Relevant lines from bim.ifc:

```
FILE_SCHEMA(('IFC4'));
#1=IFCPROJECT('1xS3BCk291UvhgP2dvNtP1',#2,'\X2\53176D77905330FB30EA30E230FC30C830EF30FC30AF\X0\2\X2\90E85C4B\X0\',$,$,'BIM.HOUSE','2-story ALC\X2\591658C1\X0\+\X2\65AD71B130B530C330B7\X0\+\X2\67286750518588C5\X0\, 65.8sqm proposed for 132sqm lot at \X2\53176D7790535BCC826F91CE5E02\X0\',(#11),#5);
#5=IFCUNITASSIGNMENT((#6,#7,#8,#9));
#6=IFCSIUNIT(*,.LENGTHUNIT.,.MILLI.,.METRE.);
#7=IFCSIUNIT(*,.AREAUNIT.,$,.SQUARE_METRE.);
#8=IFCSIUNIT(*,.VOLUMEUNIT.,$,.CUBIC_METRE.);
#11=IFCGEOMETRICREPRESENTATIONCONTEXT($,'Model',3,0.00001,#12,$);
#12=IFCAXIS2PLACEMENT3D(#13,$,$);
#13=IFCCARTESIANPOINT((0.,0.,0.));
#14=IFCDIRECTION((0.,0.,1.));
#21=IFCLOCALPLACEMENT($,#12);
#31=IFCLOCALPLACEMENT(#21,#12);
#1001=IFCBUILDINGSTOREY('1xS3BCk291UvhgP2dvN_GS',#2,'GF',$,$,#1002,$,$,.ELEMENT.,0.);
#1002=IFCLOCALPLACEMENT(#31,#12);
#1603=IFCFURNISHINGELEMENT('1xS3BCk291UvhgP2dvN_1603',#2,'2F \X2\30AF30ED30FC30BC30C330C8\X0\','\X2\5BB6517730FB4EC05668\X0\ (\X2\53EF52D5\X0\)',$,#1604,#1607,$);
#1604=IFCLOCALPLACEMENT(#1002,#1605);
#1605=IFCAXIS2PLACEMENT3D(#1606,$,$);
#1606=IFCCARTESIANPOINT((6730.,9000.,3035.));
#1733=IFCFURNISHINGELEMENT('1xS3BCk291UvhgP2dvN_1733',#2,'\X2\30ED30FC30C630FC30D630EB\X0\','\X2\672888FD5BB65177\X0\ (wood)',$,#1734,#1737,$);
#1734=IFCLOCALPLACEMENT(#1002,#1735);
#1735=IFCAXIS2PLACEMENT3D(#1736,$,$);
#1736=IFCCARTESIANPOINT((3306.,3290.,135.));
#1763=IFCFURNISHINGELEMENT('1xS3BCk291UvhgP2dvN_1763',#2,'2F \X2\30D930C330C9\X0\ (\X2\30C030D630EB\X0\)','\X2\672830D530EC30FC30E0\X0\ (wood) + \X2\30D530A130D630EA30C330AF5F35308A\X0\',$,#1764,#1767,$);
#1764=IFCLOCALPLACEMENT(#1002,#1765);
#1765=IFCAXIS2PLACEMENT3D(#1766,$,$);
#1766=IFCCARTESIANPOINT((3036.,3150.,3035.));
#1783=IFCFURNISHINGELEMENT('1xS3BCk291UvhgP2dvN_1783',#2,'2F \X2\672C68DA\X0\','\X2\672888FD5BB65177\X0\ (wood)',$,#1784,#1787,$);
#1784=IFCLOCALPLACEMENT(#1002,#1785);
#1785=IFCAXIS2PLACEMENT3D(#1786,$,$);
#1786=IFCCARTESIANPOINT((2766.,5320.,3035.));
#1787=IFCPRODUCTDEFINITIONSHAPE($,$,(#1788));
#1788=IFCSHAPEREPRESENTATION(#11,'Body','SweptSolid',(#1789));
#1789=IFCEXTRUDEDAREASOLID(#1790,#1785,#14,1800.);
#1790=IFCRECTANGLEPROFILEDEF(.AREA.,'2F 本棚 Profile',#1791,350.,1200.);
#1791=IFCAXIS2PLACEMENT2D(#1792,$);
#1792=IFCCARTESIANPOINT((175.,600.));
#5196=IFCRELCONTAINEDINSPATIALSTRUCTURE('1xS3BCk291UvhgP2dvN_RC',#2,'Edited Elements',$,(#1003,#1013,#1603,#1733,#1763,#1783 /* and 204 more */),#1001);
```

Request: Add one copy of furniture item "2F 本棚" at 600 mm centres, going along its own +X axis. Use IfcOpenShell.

```python
import ifcopenshell
import ifcopenshell.api.geometry
import ifcopenshell.api.root
import ifcopenshell.util.element
import ifcopenshell.util.placement
import ifcopenshell.util.unit

model = ifcopenshell.open("bim.ifc")
unit_scale = ifcopenshell.util.unit.calculate_unit_scale(model)


def reuse_history(source, copy):
    """copy_class also copies each property set's owner history, people and application; keep the originals."""
    for rel in copy.IsDefinedBy:
        if rel.is_a("IfcRelDefinesByProperties") and (history := rel.RelatingPropertyDefinition.OwnerHistory):
            rel.RelatingPropertyDefinition.OwnerHistory = source.OwnerHistory
            ifcopenshell.util.element.remove_deep2(model, history)


source = model.by_guid("1xS3BCk291UvhgP2dvN_1783")
base = ifcopenshell.util.placement.get_local_placement(source.ObjectPlacement)
step = base[:3, 0] * 0.6 / unit_scale

for i in range(1, 2):
    copy = ifcopenshell.api.root.copy_class(model, product=source)
    copy.Representation = ifcopenshell.util.element.copy_deep(
        model, source.Representation, exclude=["IfcGeometricRepresentationContext", "IfcRepresentationMap"]
    )
    reuse_history(source, copy)
    matrix = base.copy()
    matrix[:3, 3] += i * step
    print("added at", matrix[:3, 3].round(3) + 0.0)
    ifcopenshell.api.geometry.edit_object_placement(model, product=copy, matrix=matrix, is_si=False)

model.write("bim_rev.ifc")
```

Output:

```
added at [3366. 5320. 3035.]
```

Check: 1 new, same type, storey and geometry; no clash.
